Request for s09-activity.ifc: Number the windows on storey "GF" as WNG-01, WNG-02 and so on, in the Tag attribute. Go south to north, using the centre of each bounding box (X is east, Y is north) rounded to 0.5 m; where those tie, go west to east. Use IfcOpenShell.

First a look at what the model holds.

```python
import ifcopenshell
import ifcopenshell.util.element
import ifcopenshell.util.placement

model = ifcopenshell.open("s09-activity.ifc")
print(model.schema)
storey = next(s for s in model.by_type("IfcBuildingStorey") if s.Name == "GF")
windows = [e for e in ifcopenshell.util.element.get_decomposition(storey) if e.is_a("IfcWindow")]
for e in sorted(windows, key=lambda e: e.id()):
    origin = ifcopenshell.util.placement.get_local_placement(e.ObjectPlacement)[:3, 3]
    print(e.id(), e.Tag, e.Name, origin.round(2) + 0.0, sep=" | ")
```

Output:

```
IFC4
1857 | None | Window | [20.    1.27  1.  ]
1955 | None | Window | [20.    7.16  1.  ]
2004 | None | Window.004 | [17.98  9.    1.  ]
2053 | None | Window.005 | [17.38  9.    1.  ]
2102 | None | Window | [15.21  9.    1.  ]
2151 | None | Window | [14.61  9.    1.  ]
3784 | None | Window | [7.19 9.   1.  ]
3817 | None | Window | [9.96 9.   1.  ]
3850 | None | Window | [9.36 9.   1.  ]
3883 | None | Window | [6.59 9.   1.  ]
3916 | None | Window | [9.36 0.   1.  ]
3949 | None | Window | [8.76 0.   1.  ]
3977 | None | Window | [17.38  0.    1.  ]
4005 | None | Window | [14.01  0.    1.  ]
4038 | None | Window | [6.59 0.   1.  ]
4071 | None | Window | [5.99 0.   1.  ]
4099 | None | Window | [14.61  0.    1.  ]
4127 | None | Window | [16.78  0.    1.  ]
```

```python
import ifcopenshell
import ifcopenshell.geom
import ifcopenshell.util.element
import ifcopenshell.util.shape

model = ifcopenshell.open("s09-activity.ifc")
settings = ifcopenshell.geom.settings()
settings.set("use-world-coords", True)


def centre(element):
    shape = ifcopenshell.geom.create_shape(settings, element)
    return ifcopenshell.util.shape.get_bbox_centroid(shape.geometry)


storey = next(s for s in model.by_type("IfcBuildingStorey") if s.Name == "GF")
windows = [e for e in ifcopenshell.util.element.get_decomposition(storey) if e.is_a("IfcWindow")]

# Insertion points can sit at a corner or the storey origin, so sort by the geometry (in metres).
centres = {e: centre(e) for e in windows}
windows.sort(key=lambda e: (round(centres[e][1] / 0.5), centres[e][0]))

for i, e in enumerate(windows, start=1):
    number = f"WNG-{i:02d}"
    e.Tag = number
    print(e.id(), number)

model.write("s09-activity_edited.ifc")
```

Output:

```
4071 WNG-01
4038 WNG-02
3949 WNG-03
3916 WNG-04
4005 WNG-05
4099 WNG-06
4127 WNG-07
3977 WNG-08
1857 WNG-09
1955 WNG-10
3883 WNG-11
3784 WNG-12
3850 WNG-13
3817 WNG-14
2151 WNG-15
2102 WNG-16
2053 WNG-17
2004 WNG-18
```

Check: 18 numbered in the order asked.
